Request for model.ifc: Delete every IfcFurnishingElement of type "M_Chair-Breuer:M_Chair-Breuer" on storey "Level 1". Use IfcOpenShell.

First a look at what the model holds.

```python
import ifcopenshell
import ifcopenshell.util.element

model = ifcopenshell.open("model.ifc")
print(model.schema)
storey = next(s for s in model.by_type("IfcBuildingStorey") if s.Name == "Level 1")
furniture = [e for e in ifcopenshell.util.element.get_decomposition(storey) if e.is_a("IfcFurnishingElement")]
seen = {}
for e in furniture:
    element_type = ifcopenshell.util.element.get_type(e)
    name = element_type.Name if element_type not in (None, e) else None
    seen[name] = seen.get(name, 0) + 1
for name, count in sorted(seen.items(), key=str):
    print(count, "x", name)
```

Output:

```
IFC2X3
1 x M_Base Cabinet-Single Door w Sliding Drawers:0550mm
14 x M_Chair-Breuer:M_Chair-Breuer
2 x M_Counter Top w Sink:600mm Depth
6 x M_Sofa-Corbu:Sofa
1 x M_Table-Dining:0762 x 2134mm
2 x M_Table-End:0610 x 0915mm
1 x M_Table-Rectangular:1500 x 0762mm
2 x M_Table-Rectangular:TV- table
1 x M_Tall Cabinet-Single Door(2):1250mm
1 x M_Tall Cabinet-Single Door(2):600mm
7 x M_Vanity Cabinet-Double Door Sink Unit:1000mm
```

```python
import ifcopenshell
import ifcopenshell.api.root
import ifcopenshell.util.element

model = ifcopenshell.open("model.ifc")

storey = next(s for s in model.by_type("IfcBuildingStorey") if s.Name == "Level 1")
furniture = [e for e in ifcopenshell.util.element.get_decomposition(storey) if e.is_a("IfcFurnishingElement")]
targets = [e for e in furniture if (t := ifcopenshell.util.element.get_type(e)) not in (None, e) and t.Name == "M_Chair-Breuer:M_Chair-Breuer"]

for e in targets:
    ifcopenshell.api.root.remove_product(model, product=e)
print(len(targets), "removed")

model.write("model_updated.ifc")
```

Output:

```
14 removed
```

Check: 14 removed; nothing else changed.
